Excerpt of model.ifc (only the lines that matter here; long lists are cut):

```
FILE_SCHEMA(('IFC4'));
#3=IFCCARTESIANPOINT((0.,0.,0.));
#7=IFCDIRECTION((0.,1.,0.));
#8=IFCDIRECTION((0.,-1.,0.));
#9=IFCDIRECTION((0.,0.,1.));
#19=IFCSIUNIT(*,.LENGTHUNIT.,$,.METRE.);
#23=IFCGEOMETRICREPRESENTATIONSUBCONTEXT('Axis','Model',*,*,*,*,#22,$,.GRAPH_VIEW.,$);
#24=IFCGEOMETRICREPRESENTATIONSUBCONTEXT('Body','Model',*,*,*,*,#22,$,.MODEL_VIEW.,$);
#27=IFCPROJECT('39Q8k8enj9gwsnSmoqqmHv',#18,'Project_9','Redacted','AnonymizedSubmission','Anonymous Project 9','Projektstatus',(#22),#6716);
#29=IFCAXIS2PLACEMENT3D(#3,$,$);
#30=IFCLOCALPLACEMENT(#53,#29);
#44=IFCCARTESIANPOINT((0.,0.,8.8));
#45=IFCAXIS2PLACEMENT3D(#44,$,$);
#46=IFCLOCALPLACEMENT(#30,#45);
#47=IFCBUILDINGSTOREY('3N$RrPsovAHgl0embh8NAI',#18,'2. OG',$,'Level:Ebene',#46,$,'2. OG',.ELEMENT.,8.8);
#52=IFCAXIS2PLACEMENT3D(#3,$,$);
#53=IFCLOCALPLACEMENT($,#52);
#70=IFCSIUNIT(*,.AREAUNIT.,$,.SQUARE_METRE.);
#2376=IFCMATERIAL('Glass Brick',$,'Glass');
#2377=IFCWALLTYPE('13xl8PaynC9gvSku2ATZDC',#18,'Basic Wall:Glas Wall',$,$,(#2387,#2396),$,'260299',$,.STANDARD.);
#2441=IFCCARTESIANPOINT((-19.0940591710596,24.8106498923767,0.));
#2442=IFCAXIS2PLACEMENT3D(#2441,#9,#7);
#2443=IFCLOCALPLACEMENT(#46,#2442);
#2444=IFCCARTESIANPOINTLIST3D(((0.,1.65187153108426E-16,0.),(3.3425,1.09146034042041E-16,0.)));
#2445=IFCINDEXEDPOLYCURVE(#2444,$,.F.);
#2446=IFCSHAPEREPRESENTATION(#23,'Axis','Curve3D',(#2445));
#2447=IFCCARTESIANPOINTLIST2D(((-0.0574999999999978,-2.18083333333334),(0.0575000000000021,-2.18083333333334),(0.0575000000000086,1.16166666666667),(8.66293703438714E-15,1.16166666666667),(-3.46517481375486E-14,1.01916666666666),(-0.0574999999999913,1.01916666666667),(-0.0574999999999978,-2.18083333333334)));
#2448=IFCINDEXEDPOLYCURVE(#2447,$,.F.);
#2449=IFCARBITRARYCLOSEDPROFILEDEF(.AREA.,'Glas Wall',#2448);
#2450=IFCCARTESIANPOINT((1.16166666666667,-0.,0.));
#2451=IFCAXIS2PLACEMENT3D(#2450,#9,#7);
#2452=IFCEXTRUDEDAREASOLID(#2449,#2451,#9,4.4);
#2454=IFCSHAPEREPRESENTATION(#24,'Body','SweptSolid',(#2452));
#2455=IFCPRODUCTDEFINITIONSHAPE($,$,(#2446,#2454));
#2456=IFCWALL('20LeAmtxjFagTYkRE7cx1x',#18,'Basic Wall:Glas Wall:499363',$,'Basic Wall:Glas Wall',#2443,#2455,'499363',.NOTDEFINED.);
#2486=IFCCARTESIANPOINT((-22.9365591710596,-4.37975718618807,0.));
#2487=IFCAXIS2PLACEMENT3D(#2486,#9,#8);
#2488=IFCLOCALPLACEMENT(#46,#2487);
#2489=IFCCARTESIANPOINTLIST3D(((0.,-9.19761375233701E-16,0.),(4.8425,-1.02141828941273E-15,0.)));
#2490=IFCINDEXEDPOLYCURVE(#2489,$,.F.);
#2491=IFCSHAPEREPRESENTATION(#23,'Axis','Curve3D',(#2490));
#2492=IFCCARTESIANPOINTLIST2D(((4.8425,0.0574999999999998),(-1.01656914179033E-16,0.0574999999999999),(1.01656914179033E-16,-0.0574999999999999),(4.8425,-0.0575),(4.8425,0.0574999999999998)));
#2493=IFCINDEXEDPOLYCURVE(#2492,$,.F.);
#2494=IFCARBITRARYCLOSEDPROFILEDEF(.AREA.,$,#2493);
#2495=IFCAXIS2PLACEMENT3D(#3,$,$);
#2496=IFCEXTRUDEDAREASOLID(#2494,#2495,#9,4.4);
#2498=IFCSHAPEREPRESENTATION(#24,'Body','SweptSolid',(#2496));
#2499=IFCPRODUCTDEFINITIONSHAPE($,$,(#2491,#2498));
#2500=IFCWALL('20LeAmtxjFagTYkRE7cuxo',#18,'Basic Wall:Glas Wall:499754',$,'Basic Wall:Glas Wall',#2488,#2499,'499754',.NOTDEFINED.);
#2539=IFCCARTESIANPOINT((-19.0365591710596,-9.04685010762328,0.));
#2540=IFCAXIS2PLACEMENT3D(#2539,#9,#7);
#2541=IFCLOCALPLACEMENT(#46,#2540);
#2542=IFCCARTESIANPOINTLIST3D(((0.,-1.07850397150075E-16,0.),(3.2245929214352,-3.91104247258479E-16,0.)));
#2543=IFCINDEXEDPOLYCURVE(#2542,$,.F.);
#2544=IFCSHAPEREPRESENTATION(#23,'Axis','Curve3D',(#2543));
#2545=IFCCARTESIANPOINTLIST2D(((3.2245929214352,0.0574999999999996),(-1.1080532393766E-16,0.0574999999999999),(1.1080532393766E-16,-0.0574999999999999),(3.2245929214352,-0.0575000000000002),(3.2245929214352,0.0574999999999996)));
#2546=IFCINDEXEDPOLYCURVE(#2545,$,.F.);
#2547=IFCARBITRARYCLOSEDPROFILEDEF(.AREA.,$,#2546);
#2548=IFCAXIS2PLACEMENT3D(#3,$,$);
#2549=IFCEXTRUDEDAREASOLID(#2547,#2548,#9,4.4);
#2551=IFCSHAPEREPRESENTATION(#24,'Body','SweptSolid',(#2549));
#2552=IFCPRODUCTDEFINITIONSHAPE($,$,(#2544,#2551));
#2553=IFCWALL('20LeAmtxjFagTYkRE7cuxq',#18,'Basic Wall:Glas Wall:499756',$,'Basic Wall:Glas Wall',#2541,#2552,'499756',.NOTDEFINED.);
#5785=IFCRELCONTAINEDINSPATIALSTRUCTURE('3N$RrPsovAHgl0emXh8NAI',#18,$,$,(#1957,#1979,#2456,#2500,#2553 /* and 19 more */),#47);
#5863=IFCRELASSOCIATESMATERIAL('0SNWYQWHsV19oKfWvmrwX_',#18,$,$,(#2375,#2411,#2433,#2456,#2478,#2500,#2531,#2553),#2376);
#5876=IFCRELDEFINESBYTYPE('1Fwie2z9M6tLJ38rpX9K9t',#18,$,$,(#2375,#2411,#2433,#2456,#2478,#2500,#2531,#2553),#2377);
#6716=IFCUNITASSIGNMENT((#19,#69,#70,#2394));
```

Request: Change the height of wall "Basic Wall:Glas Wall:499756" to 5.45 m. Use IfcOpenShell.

```python
import ifcopenshell
import ifcopenshell.geom
import ifcopenshell.util.representation
import ifcopenshell.util.shape

model = ifcopenshell.open("model.ifc")
settings = ifcopenshell.geom.settings()


def volume(element):
    """Net volume in cubic metres, openings subtracted."""
    shape = ifcopenshell.geom.create_shape(settings, element)
    return ifcopenshell.util.shape.get_volume(shape.geometry)


wall = model.by_guid("20LeAmtxjFagTYkRE7cuxq")
before = volume(wall)

body = ifcopenshell.util.representation.get_representation(wall, "Model", "Body")
solid = body.Items[0]
old_height = solid.Depth
solid.Depth = 5.45
after = volume(wall)

print(f"height {old_height:g} -> {solid.Depth:g}, volume {before:.3f} -> {after:.3f} m3")

model.write("model-out.ifc")
```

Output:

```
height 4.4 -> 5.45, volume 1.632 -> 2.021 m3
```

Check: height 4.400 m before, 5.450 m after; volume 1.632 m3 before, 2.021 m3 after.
